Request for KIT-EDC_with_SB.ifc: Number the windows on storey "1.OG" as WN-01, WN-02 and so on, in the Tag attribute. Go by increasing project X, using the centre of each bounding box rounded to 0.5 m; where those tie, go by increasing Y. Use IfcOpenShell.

First a look at what the model holds.

```python
import ifcopenshell
import ifcopenshell.util.element
import ifcopenshell.util.placement

model = ifcopenshell.open("KIT-EDC_with_SB.ifc")
print(model.schema)
storey = next(s for s in model.by_type("IfcBuildingStorey") if s.Name == "1.OG")
windows = [e for e in ifcopenshell.util.element.get_decomposition(storey) if e.is_a("IfcWindow")]
for e in sorted(windows, key=lambda e: e.id()):
    origin = ifcopenshell.util.placement.get_local_placement(e.ObjectPlacement)[:3, 3]
    print(e.id(), e.Tag, e.Name, origin.round(2) + 0.0, sep=" | ")
```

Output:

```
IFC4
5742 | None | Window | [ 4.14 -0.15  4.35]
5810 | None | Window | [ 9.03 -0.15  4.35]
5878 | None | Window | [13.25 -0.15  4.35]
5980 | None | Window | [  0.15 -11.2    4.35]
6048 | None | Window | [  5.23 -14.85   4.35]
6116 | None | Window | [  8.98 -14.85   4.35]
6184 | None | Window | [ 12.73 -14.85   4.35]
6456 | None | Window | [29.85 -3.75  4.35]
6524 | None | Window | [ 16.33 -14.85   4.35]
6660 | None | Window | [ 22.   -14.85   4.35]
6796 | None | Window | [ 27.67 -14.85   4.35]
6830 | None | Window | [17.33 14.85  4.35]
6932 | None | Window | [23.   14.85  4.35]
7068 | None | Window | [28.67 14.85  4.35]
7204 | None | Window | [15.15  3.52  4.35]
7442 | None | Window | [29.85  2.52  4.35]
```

```python
import ifcopenshell
import ifcopenshell.geom
import ifcopenshell.util.element
import ifcopenshell.util.shape

model = ifcopenshell.open("KIT-EDC_with_SB.ifc")
settings = ifcopenshell.geom.settings()
settings.set("use-world-coords", True)


def centre(element):
    shape = ifcopenshell.geom.create_shape(settings, element)
    return ifcopenshell.util.shape.get_bbox_centroid(shape.geometry)


storey = next(s for s in model.by_type("IfcBuildingStorey") if s.Name == "1.OG")
windows = [e for e in ifcopenshell.util.element.get_decomposition(storey) if e.is_a("IfcWindow")]

# Insertion points can sit at a corner or the storey origin, so sort by the geometry (in metres).
centres = {e: centre(e) for e in windows}
windows.sort(key=lambda e: (round(centres[e][0] / 0.5), centres[e][1]))

for i, e in enumerate(windows, start=1):
    number = f"WN-{i:02d}"
    e.Tag = number
    print(e.id(), number)

model.write("KIT-EDC_with_SB_updated.ifc")
```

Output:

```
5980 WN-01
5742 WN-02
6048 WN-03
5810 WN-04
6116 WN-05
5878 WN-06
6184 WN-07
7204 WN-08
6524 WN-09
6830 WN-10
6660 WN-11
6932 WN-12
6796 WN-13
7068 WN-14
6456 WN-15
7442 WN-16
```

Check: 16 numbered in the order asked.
